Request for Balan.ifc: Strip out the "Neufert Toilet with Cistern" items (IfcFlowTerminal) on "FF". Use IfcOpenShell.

First a look at what the model holds.

```python
import ifcopenshell
import ifcopenshell.util.element

model = ifcopenshell.open("Balan.ifc")
print(model.schema)
storey = next(s for s in model.by_type("IfcBuildingStorey") if s.Name == "FF")
terminals = [e for e in ifcopenshell.util.element.get_decomposition(storey) if e.is_a("IfcFlowTerminal")]
seen = {}
for e in terminals:
    element_type = ifcopenshell.util.element.get_type(e)
    name = element_type.Name if element_type not in (None, e) else None
    seen[name] = seen.get(name, 0) + 1
for name, count in sorted(seen.items(), key=str):
    print(count, "x", name)
```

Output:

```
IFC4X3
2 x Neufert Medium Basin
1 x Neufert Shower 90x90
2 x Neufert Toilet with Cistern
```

```python
import ifcopenshell
import ifcopenshell.api.root
import ifcopenshell.util.element

model = ifcopenshell.open("Balan.ifc")

storey = next(s for s in model.by_type("IfcBuildingStorey") if s.Name == "FF")
terminals = [e for e in ifcopenshell.util.element.get_decomposition(storey) if e.is_a("IfcFlowTerminal")]
targets = [e for e in terminals if (t := ifcopenshell.util.element.get_type(e)) not in (None, e) and t.Name == "Neufert Toilet with Cistern"]

for e in targets:
    ifcopenshell.api.root.remove_product(model, product=e)
print(len(targets), "removed")

model.write("Balan_updated.ifc")
```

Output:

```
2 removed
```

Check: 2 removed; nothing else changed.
